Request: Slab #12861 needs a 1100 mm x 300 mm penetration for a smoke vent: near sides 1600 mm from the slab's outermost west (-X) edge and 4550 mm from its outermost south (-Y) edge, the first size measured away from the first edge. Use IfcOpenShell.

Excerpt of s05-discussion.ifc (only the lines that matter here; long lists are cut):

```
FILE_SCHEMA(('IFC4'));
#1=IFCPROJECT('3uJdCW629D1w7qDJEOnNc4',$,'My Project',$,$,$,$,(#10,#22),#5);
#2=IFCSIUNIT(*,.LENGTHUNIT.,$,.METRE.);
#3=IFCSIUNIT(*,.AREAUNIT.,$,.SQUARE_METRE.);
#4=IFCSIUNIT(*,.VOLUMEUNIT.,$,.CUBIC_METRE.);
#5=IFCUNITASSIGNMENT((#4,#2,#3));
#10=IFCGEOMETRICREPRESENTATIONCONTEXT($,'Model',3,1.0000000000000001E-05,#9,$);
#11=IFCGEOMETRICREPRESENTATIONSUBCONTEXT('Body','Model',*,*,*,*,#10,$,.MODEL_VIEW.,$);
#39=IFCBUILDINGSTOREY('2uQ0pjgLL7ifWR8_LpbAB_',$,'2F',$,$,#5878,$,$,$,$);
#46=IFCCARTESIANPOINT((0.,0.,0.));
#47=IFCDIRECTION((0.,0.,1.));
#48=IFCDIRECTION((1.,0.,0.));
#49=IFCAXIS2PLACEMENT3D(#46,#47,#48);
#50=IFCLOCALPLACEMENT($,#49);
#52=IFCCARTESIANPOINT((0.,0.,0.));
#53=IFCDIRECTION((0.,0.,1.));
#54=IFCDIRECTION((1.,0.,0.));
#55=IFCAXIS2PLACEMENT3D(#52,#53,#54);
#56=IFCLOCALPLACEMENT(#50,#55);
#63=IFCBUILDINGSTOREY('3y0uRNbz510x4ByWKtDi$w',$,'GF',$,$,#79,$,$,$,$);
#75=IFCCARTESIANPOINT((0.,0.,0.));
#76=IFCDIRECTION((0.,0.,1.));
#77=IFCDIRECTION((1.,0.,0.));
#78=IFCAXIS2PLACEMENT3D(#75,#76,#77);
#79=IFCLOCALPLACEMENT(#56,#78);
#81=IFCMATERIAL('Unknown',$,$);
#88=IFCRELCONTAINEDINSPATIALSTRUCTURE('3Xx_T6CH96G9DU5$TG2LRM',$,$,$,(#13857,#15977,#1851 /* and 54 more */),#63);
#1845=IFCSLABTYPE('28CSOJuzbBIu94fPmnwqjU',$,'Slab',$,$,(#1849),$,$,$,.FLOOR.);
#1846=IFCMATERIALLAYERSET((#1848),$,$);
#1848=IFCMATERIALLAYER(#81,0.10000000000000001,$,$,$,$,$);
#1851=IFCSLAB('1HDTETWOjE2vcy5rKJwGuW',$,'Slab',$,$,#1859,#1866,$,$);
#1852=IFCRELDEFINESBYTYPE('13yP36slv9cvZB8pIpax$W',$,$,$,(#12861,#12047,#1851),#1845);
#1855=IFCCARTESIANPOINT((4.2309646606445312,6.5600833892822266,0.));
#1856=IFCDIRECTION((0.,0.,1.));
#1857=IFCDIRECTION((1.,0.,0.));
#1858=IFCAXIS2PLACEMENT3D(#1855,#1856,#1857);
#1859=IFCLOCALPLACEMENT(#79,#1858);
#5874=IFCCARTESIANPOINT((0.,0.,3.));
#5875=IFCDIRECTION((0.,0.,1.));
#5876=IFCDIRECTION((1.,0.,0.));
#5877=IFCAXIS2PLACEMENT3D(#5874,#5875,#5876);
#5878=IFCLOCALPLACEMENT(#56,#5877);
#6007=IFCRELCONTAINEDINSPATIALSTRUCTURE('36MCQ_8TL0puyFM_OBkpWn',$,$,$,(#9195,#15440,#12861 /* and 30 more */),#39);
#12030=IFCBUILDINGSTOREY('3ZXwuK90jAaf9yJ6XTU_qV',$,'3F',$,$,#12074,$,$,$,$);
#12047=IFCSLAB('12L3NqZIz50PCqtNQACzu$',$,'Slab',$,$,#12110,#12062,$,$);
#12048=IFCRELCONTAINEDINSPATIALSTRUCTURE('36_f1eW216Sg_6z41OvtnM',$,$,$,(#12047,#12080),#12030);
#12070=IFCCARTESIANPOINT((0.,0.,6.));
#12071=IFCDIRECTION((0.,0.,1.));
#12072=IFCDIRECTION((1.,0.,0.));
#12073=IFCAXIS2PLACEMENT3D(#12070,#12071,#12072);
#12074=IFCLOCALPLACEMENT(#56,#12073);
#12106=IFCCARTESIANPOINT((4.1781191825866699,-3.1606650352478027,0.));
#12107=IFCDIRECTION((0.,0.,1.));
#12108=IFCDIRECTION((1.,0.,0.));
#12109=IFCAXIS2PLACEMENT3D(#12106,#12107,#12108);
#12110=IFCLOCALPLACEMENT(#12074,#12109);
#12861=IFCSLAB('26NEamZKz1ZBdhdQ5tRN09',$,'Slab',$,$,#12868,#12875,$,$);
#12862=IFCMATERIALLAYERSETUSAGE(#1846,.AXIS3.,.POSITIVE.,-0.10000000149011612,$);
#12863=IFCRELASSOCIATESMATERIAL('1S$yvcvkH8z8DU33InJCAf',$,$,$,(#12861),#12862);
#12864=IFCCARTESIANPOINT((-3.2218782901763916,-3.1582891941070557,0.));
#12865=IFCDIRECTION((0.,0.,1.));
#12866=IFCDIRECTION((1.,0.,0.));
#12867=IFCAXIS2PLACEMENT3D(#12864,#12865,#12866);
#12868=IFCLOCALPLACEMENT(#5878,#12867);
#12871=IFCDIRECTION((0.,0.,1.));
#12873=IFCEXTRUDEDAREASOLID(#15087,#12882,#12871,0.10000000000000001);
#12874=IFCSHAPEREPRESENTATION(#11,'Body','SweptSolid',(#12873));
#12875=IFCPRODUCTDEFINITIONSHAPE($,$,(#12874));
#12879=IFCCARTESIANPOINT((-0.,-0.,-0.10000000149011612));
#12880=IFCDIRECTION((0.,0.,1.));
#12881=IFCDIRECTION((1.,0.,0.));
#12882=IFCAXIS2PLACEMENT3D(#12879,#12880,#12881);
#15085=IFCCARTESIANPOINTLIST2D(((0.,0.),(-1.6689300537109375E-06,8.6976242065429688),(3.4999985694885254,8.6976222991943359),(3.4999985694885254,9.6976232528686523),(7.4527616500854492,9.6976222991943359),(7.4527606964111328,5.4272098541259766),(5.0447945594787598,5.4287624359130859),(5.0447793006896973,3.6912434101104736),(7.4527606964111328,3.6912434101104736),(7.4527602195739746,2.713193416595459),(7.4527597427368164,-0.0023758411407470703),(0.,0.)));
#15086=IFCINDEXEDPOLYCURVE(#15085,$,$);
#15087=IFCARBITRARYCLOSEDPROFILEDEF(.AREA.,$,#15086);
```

```python
import numpy as np
import ifcopenshell
import ifcopenshell.api.feature
import ifcopenshell.api.geometry
import ifcopenshell.api.root
import ifcopenshell.geom
import ifcopenshell.util.placement
import ifcopenshell.util.representation
import ifcopenshell.util.shape
import ifcopenshell.util.unit

model = ifcopenshell.open("s05-discussion.ifc")
unit_scale = ifcopenshell.util.unit.calculate_unit_scale(model)
settings = ifcopenshell.geom.settings()


def volume(element):
    """Net volume in cubic metres, openings subtracted."""
    shape = ifcopenshell.geom.create_shape(settings, element)
    return ifcopenshell.util.shape.get_volume(shape.geometry)


slab = model.by_id(12861)
before = volume(slab)

# Extent in the slab's own axes, in metres. The edges named are its -X and -Y sides.
slab_shape = ifcopenshell.geom.create_shape(settings, slab)
vertices = ifcopenshell.util.shape.get_vertices(slab_shape.geometry)
x_min, y_min, bottom = vertices.min(axis=0)
top = vertices[:, 2].max()

opening = ifcopenshell.api.root.create_entity(model, ifc_class="IfcOpeningElement", name="Smoke vent opening", predefined_type="OPENING")
context = ifcopenshell.util.representation.get_context(model, "Model", "Body", "MODEL_VIEW")
width, depth = 1.1, 0.3
outline = [(0.0, 0.0), (width, 0.0), (width, depth), (0.0, depth), (0.0, 0.0)]
# Overshoot both faces by 50 mm so the cut is clean.
shape = ifcopenshell.api.geometry.add_slab_representation(
    model, context=context, depth=top - bottom + 0.1, polyline=outline
)
ifcopenshell.api.geometry.assign_representation(model, product=opening, representation=shape)

matrix = ifcopenshell.util.placement.get_local_placement(slab.ObjectPlacement)
matrix[:, 3] = matrix @ np.append(np.array([x_min + 1.6, y_min + 4.55, bottom - 0.05]) / unit_scale, 1.0)
ifcopenshell.api.geometry.edit_object_placement(model, product=opening, matrix=matrix, is_si=False)
ifcopenshell.api.feature.add_feature(model, feature=opening, element=slab)

after = volume(slab)

print(f"slab volume {before:.3f} -> {after:.3f} m3")

model.write("s05-discussion_rev.ifc")
```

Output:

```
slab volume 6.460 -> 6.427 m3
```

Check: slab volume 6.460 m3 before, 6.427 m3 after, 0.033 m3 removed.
